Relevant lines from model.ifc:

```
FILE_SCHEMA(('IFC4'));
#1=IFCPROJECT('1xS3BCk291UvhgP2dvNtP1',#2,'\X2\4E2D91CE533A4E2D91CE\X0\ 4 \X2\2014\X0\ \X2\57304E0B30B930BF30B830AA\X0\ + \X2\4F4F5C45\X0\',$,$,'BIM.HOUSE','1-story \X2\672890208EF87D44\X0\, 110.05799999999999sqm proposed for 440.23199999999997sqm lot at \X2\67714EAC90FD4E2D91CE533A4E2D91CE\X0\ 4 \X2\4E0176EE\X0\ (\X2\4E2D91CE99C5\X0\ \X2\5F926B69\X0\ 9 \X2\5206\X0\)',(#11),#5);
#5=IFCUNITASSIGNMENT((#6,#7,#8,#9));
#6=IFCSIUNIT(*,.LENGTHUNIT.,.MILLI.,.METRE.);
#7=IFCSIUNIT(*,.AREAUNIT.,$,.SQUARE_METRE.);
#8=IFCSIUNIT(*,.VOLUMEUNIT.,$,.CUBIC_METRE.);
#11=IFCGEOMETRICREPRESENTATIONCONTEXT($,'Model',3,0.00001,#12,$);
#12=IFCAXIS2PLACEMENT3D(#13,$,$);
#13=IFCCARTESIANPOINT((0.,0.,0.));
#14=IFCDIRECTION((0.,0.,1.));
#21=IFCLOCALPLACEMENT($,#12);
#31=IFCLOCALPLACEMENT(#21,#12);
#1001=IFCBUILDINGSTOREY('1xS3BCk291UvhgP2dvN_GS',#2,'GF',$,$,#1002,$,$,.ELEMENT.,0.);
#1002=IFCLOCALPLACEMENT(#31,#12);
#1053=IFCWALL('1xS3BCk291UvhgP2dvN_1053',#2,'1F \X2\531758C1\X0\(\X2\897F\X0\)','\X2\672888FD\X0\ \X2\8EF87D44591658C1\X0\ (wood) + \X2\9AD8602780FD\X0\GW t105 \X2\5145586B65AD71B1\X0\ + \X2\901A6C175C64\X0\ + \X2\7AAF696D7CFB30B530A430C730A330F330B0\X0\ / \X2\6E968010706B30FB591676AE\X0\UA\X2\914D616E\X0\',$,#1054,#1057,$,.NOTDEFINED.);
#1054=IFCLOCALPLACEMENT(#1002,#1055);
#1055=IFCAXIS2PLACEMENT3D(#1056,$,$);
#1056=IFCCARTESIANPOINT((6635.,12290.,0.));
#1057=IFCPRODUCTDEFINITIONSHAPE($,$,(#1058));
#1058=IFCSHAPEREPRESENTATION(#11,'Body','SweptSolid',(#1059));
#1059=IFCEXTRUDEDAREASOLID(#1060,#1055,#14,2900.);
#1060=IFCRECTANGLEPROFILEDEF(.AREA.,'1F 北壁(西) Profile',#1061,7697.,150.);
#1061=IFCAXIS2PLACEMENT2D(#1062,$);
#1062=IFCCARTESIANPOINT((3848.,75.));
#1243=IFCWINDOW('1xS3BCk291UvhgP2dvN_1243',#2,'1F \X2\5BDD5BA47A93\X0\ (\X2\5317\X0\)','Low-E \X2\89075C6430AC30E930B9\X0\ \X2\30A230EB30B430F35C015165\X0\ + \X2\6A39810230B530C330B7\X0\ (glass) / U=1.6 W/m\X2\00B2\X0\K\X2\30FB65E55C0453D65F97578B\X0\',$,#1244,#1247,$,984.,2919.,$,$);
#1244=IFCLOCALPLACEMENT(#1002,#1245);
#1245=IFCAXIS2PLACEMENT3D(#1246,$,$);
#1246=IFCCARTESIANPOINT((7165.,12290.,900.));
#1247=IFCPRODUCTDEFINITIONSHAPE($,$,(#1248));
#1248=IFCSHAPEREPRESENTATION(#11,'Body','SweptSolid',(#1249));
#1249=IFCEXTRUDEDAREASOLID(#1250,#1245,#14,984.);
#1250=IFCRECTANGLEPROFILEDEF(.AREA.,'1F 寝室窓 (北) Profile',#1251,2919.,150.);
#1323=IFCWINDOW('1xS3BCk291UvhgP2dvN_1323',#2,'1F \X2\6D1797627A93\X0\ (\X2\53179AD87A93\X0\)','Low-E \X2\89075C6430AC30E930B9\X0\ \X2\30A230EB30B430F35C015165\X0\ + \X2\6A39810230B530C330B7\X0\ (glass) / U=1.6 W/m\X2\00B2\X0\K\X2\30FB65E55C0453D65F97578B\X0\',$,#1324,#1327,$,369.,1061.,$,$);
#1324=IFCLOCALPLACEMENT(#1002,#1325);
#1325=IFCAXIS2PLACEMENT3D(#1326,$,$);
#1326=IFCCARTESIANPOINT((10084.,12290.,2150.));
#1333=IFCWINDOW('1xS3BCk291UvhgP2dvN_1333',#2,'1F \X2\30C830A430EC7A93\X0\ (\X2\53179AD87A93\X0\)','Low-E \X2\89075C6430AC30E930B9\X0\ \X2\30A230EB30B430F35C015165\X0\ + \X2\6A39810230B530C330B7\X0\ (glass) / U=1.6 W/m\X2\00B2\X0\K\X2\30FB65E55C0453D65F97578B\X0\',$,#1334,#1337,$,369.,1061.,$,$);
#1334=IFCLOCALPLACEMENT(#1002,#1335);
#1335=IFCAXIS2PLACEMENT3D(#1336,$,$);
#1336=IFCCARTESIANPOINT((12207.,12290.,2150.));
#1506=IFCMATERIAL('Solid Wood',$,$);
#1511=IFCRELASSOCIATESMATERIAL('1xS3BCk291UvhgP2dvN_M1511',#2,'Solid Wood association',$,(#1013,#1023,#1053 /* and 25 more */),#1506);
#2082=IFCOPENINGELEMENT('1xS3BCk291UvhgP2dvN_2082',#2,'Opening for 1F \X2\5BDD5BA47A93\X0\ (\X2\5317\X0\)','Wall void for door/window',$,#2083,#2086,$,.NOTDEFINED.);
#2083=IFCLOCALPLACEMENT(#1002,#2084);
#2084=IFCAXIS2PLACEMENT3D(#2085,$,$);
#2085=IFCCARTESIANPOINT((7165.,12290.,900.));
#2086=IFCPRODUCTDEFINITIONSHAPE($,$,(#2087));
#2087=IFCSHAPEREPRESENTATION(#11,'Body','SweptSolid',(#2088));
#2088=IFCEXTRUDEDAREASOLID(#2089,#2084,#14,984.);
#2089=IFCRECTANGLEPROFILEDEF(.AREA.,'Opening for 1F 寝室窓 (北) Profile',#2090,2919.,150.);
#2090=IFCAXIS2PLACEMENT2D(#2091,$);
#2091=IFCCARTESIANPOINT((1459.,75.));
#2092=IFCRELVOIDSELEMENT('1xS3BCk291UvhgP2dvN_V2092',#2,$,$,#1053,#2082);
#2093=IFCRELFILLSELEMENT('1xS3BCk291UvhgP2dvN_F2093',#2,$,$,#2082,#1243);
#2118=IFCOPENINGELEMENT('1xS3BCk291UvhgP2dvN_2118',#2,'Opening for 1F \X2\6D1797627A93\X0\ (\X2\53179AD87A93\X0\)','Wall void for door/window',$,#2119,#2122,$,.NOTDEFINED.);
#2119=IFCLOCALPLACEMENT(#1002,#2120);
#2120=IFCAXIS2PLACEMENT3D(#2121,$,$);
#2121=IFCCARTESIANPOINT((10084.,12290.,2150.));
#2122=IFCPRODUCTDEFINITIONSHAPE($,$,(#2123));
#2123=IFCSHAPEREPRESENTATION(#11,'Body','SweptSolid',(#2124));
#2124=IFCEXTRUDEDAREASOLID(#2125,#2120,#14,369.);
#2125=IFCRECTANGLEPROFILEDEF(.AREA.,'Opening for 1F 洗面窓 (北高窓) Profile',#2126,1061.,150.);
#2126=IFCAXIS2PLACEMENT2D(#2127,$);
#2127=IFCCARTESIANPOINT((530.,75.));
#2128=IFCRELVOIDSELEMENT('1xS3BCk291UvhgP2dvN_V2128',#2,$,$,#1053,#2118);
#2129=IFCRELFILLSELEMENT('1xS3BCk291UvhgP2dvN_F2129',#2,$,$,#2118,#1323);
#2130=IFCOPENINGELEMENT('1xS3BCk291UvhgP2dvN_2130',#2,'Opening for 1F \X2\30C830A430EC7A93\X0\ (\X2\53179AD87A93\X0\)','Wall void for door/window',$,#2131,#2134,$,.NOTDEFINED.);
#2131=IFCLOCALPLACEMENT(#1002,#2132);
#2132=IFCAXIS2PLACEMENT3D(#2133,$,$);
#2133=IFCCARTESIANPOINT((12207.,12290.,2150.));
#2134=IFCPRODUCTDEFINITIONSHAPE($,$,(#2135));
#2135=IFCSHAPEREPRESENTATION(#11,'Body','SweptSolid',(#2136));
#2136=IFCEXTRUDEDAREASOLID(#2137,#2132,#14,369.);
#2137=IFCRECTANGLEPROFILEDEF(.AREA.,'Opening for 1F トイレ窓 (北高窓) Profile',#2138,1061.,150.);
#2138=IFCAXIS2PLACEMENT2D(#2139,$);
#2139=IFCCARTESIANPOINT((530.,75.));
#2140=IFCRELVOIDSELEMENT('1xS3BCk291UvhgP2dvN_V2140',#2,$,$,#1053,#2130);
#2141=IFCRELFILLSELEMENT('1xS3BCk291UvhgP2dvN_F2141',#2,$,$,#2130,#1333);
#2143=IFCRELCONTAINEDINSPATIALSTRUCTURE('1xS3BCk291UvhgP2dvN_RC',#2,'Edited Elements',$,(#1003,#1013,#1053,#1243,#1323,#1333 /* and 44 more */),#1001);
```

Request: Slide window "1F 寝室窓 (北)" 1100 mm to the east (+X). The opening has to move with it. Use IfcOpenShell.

```python
import ifcopenshell
import ifcopenshell.api.geometry
import ifcopenshell.util.placement

model = ifcopenshell.open("model.ifc")

window = model.by_id(1243)
opening = window.FillsVoids[0].RelatingOpeningElement
wall = opening.VoidsElements[0].RelatingBuildingElement

wall_matrix = ifcopenshell.util.placement.get_local_placement(wall.ObjectPlacement)
shift = wall_matrix[:3, 0] * 1100.0
before = ifcopenshell.util.placement.get_local_placement(window.ObjectPlacement)[:3, 3].copy()

# The window is not placed relative to its opening, so move both.
for product in (opening, window):
    matrix = ifcopenshell.util.placement.get_local_placement(product.ObjectPlacement)
    matrix[:3, 3] += shift
    ifcopenshell.api.geometry.edit_object_placement(model, product=product, matrix=matrix, is_si=False)

after = ifcopenshell.util.placement.get_local_placement(window.ObjectPlacement)[:3, 3]
print("window moved by", (after - before).round(3) + 0.0)

model.write("model_edited.ifc")
```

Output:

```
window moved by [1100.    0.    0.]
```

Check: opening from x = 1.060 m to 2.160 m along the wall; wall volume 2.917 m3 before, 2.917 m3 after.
